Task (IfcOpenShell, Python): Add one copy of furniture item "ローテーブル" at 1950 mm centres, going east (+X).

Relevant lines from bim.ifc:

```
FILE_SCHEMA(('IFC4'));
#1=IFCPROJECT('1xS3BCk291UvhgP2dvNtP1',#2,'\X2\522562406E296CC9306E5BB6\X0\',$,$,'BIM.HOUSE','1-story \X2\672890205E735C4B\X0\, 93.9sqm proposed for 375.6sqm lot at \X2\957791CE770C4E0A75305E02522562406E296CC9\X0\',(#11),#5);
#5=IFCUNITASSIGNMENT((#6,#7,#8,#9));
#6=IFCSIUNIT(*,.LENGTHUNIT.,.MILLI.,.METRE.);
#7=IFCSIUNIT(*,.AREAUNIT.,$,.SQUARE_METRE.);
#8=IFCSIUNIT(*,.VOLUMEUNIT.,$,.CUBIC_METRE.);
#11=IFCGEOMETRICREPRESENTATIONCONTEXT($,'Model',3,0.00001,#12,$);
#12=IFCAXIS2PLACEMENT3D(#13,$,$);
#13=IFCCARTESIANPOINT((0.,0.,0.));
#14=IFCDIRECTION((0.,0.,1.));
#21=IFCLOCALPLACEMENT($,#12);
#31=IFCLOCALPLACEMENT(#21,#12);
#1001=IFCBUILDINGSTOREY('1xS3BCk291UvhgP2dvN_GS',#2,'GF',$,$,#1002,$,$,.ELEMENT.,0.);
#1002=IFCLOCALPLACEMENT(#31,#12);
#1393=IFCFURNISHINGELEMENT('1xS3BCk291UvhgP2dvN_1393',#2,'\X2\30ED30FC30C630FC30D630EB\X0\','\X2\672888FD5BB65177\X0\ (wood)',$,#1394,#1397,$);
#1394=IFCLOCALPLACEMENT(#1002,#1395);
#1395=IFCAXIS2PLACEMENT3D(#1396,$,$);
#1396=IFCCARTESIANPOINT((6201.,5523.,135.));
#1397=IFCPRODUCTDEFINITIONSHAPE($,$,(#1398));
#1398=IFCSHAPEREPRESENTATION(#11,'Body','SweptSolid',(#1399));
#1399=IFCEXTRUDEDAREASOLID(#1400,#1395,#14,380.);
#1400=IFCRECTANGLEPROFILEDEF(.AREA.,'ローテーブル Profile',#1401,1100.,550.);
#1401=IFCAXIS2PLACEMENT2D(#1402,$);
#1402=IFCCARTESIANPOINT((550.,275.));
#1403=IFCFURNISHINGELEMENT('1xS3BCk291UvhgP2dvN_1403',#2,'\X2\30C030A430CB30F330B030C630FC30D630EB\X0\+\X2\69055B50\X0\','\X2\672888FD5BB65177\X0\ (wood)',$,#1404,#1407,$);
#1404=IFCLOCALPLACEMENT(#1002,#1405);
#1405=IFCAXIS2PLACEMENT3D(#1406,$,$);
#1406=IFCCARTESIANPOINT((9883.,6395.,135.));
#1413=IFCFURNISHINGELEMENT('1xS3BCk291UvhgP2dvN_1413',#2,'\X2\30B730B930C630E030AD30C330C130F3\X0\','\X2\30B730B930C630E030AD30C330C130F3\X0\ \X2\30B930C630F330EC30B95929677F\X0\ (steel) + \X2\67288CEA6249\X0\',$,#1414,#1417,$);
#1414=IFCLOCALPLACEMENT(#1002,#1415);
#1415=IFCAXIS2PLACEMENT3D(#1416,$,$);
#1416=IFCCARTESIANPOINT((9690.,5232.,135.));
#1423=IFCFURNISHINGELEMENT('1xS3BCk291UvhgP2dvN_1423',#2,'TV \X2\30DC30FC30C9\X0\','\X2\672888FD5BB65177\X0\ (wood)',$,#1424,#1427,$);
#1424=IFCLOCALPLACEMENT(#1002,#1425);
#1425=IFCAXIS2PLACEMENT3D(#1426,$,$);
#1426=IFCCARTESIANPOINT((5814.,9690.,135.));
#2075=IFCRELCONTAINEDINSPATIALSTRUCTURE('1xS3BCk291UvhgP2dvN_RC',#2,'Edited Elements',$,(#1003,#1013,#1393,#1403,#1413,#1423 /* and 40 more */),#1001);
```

```python
import numpy as np
import ifcopenshell
import ifcopenshell.api.geometry
import ifcopenshell.api.root
import ifcopenshell.util.element
import ifcopenshell.util.placement
import ifcopenshell.util.unit

model = ifcopenshell.open("bim.ifc")
unit_scale = ifcopenshell.util.unit.calculate_unit_scale(model)


def reuse_history(source, copy):
    """copy_class also copies each property set's owner history, people and application; keep the originals."""
    for rel in copy.IsDefinedBy:
        if rel.is_a("IfcRelDefinesByProperties") and (history := rel.RelatingPropertyDefinition.OwnerHistory):
            rel.RelatingPropertyDefinition.OwnerHistory = source.OwnerHistory
            ifcopenshell.util.element.remove_deep2(model, history)


source = model.by_guid("1xS3BCk291UvhgP2dvN_1393")
base = ifcopenshell.util.placement.get_local_placement(source.ObjectPlacement)
step = np.array([1.0, 0.0, 0.0]) * 1.95 / unit_scale

for i in range(1, 2):
    copy = ifcopenshell.api.root.copy_class(model, product=source)
    copy.Representation = ifcopenshell.util.element.copy_deep(
        model, source.Representation, exclude=["IfcGeometricRepresentationContext", "IfcRepresentationMap"]
    )
    reuse_history(source, copy)
    matrix = base.copy()
    matrix[:3, 3] += i * step
    print("added at", matrix[:3, 3].round(3) + 0.0)
    ifcopenshell.api.geometry.edit_object_placement(model, product=copy, matrix=matrix, is_si=False)

model.write("bim_v2.ifc")
```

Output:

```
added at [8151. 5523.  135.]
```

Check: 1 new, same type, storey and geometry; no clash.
